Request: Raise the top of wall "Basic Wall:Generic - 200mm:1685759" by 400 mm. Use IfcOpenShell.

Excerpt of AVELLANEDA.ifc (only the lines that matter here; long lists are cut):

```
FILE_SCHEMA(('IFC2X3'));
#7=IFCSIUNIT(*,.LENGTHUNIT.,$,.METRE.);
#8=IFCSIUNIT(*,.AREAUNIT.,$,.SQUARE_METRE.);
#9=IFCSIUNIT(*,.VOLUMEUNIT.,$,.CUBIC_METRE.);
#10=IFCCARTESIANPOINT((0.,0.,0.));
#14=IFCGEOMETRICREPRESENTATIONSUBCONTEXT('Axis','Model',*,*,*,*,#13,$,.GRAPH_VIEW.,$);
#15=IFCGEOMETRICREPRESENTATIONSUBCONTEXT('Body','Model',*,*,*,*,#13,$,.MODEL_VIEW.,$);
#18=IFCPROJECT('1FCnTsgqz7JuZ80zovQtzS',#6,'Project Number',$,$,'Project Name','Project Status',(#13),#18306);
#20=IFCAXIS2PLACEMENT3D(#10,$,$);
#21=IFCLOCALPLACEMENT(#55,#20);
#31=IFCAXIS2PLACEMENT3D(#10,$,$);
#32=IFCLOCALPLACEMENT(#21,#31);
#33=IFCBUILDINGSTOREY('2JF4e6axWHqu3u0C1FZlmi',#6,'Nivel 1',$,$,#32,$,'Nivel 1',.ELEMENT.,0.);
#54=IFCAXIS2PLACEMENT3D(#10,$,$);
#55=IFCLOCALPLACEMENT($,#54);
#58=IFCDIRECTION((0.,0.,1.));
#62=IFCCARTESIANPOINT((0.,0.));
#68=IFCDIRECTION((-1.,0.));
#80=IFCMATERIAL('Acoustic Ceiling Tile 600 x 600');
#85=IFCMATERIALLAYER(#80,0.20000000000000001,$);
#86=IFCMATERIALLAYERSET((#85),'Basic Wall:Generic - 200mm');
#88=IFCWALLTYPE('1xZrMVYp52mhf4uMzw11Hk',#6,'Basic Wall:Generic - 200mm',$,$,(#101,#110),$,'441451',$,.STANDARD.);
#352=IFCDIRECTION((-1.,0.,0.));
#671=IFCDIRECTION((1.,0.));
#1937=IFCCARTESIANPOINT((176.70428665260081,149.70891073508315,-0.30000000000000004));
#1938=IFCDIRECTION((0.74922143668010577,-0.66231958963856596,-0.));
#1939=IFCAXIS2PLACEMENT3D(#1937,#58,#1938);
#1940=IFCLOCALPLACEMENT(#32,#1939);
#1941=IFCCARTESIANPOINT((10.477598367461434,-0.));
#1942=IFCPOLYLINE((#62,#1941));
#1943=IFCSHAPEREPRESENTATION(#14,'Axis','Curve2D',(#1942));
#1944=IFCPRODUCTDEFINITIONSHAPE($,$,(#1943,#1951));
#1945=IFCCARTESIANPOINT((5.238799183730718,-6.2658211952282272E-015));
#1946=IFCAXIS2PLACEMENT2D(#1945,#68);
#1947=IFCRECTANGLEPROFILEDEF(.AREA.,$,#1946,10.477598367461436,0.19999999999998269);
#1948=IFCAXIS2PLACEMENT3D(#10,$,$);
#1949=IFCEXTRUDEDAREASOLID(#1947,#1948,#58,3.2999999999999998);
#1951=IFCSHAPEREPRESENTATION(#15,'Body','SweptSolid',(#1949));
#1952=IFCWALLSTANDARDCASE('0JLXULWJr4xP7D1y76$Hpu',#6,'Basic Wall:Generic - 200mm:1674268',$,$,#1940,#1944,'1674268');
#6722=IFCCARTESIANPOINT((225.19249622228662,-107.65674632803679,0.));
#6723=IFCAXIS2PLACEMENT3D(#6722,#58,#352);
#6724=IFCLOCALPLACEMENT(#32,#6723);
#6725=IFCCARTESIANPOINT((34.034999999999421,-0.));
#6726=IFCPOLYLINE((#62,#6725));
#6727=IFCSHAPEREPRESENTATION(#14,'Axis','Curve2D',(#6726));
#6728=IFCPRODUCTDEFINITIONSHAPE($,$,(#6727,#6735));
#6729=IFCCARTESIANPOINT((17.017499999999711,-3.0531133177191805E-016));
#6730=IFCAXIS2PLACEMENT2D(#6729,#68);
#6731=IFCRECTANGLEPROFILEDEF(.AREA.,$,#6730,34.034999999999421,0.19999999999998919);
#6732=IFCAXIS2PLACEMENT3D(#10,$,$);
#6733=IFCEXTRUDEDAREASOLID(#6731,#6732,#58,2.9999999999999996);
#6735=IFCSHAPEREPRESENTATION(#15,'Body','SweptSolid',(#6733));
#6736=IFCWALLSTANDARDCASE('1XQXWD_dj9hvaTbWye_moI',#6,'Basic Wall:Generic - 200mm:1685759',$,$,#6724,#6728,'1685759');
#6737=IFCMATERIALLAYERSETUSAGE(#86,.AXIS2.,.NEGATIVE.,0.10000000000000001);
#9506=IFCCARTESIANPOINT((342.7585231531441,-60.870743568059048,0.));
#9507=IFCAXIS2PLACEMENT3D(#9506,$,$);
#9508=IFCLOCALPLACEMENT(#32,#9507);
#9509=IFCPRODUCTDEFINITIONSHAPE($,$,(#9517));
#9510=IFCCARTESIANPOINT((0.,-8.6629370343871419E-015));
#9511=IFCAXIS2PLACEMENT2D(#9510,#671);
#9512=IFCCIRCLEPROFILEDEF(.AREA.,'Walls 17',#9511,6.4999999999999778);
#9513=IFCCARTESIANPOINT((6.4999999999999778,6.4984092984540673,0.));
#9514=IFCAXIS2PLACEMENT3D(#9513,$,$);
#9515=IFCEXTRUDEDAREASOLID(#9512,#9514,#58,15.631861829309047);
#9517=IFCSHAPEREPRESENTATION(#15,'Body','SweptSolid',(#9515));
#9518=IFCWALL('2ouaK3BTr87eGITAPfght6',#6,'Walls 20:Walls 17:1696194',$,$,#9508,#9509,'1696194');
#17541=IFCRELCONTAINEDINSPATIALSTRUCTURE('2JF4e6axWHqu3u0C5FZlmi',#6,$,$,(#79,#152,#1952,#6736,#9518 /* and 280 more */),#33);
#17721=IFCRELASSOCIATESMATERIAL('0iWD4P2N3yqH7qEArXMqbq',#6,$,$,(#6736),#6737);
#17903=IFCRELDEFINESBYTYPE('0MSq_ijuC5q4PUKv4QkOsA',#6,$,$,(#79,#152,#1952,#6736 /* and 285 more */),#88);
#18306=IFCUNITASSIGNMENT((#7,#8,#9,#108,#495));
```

```python
import ifcopenshell
import ifcopenshell.geom
import ifcopenshell.util.representation
import ifcopenshell.util.shape
import ifcopenshell.util.unit

model = ifcopenshell.open("AVELLANEDA.ifc")
unit_scale = ifcopenshell.util.unit.calculate_unit_scale(model)
settings = ifcopenshell.geom.settings()


def volume(element):
    """Net volume in cubic metres, openings subtracted."""
    shape = ifcopenshell.geom.create_shape(settings, element)
    return ifcopenshell.util.shape.get_volume(shape.geometry)


wall = model.by_guid("1XQXWD_dj9hvaTbWye_moI")
before = volume(wall)

body = ifcopenshell.util.representation.get_representation(wall, "Model", "Body")
solid = body.Items[0]
old_height = solid.Depth
solid.Depth += 0.4 / unit_scale
after = volume(wall)

print(f"height {old_height:g} -> {solid.Depth:g}, volume {before:.3f} -> {after:.3f} m3")

model.write("AVELLANEDA_rev.ifc")
```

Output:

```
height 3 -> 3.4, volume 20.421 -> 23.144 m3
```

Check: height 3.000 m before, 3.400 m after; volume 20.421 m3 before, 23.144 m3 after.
